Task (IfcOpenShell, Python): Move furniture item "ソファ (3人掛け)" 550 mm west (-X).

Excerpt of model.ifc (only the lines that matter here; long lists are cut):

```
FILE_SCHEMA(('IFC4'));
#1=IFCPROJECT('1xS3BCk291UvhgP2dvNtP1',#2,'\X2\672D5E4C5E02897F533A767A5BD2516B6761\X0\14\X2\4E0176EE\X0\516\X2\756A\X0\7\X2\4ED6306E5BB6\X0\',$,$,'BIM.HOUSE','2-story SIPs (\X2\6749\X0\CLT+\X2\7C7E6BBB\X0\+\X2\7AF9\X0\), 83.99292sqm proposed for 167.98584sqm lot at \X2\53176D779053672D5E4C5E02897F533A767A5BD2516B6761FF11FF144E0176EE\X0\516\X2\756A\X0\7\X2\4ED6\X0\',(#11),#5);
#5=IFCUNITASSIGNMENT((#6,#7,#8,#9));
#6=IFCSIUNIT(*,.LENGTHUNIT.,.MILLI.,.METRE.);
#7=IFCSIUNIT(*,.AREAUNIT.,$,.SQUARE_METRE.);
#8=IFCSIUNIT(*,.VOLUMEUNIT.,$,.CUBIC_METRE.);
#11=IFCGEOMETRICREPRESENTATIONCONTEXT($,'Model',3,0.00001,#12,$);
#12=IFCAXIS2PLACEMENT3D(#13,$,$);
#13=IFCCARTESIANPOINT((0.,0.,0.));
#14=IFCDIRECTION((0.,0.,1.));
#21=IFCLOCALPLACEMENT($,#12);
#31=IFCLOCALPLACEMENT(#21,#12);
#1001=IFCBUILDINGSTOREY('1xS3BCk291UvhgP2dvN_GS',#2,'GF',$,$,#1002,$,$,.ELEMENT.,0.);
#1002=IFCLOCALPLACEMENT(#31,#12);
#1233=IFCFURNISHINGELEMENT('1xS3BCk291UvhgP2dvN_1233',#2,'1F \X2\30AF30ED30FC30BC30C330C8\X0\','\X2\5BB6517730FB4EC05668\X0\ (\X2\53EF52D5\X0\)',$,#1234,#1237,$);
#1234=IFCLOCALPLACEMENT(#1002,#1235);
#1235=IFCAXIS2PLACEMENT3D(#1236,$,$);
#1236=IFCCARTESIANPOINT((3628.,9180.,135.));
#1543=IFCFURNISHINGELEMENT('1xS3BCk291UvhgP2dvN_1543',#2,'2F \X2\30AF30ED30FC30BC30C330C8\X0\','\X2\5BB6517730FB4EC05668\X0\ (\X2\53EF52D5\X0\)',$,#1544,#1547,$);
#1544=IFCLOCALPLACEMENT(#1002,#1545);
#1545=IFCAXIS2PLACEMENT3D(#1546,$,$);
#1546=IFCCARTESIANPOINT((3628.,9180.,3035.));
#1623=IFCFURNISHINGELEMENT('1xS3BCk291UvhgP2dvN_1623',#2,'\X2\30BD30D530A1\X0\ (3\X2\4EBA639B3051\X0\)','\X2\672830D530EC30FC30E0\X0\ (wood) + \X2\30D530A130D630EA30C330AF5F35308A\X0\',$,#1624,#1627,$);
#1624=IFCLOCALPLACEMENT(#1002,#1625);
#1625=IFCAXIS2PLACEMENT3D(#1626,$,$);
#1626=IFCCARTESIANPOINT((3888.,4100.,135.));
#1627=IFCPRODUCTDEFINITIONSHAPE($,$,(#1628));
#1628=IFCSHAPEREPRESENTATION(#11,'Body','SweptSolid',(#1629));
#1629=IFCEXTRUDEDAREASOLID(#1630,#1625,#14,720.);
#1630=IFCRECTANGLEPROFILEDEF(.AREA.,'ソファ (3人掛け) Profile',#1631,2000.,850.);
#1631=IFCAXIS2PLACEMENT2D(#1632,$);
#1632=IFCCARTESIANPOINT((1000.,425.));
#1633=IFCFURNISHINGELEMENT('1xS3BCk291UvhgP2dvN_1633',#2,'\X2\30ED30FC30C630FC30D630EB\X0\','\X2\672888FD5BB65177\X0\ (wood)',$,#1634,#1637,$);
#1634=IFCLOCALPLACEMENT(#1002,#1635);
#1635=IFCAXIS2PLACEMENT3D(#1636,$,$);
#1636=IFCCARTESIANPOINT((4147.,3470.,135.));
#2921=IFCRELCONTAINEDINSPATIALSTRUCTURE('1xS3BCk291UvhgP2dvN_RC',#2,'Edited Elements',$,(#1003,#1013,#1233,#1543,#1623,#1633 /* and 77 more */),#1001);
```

```python
import ifcopenshell
import ifcopenshell.api.geometry
import ifcopenshell.util.placement
import ifcopenshell.util.unit

model = ifcopenshell.open("model.ifc")
unit_scale = ifcopenshell.util.unit.calculate_unit_scale(model)

item = model.by_guid("1xS3BCk291UvhgP2dvN_1623")
matrix = ifcopenshell.util.placement.get_local_placement(item.ObjectPlacement)
matrix[0, 3] -= 0.55 / unit_scale
ifcopenshell.api.geometry.edit_object_placement(model, product=item, matrix=matrix, is_si=False)

print(ifcopenshell.util.placement.get_local_placement(item.ObjectPlacement).round(3) + 0.0)

model.write("model_rev.ifc")
```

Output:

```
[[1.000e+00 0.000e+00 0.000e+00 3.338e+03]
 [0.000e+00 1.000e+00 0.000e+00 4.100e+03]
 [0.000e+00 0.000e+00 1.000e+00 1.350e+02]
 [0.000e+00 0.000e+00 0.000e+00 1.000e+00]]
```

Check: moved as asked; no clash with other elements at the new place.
